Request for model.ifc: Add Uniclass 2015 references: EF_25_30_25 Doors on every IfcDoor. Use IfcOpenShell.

First a look at what the model holds.

```python
import ifcopenshell

model = ifcopenshell.open("model.ifc")
print(model.schema)
print("classifications:", [c.Name for c in model.by_type("IfcClassification")])
for ifc_class in ("IfcDoor", "IfcRoof", "IfcStair", "IfcWall", "IfcWindow"):
    print(ifc_class, len(model.by_type(ifc_class)))
```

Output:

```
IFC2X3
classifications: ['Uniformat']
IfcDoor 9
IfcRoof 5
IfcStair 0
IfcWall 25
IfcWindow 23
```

```python
import ifcopenshell
import ifcopenshell.api.classification

model = ifcopenshell.open("model.ifc")

# IFC2X3 requires Source and Edition and has no link from the project to the system.
system = model.create_entity("IfcClassification", Source="NBS", Edition="2015", Name="Uniclass 2015")

codes = {
    "IfcDoor": ("EF_25_30_25", "Doors"),
}
for ifc_class, (code, name) in codes.items():
    products = model.by_type(ifc_class)
    ifcopenshell.api.classification.add_reference(
        model, products=products, classification=system, identification=code, name=name
    )
    print(code, len(products))

model.write("model_rev.ifc")
```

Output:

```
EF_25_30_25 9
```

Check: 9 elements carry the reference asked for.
